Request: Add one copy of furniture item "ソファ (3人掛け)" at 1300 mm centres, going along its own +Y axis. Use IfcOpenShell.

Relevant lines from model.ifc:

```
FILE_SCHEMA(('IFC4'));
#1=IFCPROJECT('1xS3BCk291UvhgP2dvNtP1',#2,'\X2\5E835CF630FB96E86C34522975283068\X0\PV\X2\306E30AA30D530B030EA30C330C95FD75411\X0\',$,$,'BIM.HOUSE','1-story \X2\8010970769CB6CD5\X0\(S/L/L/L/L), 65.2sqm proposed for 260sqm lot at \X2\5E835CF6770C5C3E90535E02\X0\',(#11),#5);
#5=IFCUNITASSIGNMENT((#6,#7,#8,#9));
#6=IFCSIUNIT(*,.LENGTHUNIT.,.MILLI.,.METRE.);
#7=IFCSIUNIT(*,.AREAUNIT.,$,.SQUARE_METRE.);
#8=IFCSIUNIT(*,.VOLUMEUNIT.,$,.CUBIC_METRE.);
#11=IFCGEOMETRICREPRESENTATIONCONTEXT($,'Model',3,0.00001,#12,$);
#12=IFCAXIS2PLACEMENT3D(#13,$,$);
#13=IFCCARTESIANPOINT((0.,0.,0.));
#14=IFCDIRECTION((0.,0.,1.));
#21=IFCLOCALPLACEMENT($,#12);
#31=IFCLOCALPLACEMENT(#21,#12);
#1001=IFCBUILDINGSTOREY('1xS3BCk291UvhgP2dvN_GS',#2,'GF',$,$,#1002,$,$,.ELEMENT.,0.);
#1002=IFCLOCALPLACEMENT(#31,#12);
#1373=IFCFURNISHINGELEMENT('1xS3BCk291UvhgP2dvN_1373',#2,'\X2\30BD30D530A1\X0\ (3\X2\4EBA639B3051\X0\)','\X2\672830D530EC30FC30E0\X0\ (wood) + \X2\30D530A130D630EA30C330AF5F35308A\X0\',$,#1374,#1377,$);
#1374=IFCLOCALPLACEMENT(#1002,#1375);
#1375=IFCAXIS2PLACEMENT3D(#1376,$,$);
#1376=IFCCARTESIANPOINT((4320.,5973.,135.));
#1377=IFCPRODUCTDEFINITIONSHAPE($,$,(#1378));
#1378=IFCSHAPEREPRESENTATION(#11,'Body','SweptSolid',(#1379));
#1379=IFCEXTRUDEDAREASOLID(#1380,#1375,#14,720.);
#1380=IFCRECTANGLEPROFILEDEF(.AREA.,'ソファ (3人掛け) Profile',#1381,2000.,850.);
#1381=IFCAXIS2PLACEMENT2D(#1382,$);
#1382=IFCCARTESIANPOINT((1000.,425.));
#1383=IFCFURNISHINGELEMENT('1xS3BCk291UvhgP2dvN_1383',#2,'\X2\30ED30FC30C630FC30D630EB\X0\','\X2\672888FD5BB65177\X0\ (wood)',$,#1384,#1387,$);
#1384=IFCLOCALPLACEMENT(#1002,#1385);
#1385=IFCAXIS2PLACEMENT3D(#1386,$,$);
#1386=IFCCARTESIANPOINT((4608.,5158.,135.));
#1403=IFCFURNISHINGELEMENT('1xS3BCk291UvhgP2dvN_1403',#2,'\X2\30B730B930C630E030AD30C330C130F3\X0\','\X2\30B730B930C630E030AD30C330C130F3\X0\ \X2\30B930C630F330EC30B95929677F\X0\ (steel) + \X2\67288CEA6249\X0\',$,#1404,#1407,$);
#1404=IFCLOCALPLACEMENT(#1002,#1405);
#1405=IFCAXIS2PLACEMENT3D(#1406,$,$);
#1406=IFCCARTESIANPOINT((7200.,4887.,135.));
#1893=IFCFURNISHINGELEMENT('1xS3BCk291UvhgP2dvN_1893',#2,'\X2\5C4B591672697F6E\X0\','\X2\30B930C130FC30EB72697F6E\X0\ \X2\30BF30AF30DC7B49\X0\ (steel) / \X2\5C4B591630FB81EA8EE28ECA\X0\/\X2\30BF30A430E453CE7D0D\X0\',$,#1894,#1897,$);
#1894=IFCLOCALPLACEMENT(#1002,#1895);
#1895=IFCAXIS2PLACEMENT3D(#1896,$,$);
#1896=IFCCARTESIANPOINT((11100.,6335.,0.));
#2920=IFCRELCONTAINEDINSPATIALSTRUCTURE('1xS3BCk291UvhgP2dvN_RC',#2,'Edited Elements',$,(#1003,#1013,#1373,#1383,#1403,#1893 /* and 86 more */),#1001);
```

```python
import ifcopenshell
import ifcopenshell.api.geometry
import ifcopenshell.api.root
import ifcopenshell.util.element
import ifcopenshell.util.placement

model = ifcopenshell.open("model.ifc")


def reuse_history(source, copy):
    """copy_class also copies each property set's owner history, people and application; keep the originals."""
    for rel in copy.IsDefinedBy:
        if rel.is_a("IfcRelDefinesByProperties") and (history := rel.RelatingPropertyDefinition.OwnerHistory):
            rel.RelatingPropertyDefinition.OwnerHistory = source.OwnerHistory
            ifcopenshell.util.element.remove_deep2(model, history)


source = model.by_guid("1xS3BCk291UvhgP2dvN_1373")
base = ifcopenshell.util.placement.get_local_placement(source.ObjectPlacement)
step = base[:3, 1] * 1300.0

for i in range(1, 2):
    copy = ifcopenshell.api.root.copy_class(model, product=source)
    copy.Representation = ifcopenshell.util.element.copy_deep(
        model, source.Representation, exclude=["IfcGeometricRepresentationContext", "IfcRepresentationMap"]
    )
    reuse_history(source, copy)
    matrix = base.copy()
    matrix[:3, 3] += i * step
    print("added at", matrix[:3, 3].round(3) + 0.0)
    ifcopenshell.api.geometry.edit_object_placement(model, product=copy, matrix=matrix, is_si=False)

model.write("model_edited.ifc")
```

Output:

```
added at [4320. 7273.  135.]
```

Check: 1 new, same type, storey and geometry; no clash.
